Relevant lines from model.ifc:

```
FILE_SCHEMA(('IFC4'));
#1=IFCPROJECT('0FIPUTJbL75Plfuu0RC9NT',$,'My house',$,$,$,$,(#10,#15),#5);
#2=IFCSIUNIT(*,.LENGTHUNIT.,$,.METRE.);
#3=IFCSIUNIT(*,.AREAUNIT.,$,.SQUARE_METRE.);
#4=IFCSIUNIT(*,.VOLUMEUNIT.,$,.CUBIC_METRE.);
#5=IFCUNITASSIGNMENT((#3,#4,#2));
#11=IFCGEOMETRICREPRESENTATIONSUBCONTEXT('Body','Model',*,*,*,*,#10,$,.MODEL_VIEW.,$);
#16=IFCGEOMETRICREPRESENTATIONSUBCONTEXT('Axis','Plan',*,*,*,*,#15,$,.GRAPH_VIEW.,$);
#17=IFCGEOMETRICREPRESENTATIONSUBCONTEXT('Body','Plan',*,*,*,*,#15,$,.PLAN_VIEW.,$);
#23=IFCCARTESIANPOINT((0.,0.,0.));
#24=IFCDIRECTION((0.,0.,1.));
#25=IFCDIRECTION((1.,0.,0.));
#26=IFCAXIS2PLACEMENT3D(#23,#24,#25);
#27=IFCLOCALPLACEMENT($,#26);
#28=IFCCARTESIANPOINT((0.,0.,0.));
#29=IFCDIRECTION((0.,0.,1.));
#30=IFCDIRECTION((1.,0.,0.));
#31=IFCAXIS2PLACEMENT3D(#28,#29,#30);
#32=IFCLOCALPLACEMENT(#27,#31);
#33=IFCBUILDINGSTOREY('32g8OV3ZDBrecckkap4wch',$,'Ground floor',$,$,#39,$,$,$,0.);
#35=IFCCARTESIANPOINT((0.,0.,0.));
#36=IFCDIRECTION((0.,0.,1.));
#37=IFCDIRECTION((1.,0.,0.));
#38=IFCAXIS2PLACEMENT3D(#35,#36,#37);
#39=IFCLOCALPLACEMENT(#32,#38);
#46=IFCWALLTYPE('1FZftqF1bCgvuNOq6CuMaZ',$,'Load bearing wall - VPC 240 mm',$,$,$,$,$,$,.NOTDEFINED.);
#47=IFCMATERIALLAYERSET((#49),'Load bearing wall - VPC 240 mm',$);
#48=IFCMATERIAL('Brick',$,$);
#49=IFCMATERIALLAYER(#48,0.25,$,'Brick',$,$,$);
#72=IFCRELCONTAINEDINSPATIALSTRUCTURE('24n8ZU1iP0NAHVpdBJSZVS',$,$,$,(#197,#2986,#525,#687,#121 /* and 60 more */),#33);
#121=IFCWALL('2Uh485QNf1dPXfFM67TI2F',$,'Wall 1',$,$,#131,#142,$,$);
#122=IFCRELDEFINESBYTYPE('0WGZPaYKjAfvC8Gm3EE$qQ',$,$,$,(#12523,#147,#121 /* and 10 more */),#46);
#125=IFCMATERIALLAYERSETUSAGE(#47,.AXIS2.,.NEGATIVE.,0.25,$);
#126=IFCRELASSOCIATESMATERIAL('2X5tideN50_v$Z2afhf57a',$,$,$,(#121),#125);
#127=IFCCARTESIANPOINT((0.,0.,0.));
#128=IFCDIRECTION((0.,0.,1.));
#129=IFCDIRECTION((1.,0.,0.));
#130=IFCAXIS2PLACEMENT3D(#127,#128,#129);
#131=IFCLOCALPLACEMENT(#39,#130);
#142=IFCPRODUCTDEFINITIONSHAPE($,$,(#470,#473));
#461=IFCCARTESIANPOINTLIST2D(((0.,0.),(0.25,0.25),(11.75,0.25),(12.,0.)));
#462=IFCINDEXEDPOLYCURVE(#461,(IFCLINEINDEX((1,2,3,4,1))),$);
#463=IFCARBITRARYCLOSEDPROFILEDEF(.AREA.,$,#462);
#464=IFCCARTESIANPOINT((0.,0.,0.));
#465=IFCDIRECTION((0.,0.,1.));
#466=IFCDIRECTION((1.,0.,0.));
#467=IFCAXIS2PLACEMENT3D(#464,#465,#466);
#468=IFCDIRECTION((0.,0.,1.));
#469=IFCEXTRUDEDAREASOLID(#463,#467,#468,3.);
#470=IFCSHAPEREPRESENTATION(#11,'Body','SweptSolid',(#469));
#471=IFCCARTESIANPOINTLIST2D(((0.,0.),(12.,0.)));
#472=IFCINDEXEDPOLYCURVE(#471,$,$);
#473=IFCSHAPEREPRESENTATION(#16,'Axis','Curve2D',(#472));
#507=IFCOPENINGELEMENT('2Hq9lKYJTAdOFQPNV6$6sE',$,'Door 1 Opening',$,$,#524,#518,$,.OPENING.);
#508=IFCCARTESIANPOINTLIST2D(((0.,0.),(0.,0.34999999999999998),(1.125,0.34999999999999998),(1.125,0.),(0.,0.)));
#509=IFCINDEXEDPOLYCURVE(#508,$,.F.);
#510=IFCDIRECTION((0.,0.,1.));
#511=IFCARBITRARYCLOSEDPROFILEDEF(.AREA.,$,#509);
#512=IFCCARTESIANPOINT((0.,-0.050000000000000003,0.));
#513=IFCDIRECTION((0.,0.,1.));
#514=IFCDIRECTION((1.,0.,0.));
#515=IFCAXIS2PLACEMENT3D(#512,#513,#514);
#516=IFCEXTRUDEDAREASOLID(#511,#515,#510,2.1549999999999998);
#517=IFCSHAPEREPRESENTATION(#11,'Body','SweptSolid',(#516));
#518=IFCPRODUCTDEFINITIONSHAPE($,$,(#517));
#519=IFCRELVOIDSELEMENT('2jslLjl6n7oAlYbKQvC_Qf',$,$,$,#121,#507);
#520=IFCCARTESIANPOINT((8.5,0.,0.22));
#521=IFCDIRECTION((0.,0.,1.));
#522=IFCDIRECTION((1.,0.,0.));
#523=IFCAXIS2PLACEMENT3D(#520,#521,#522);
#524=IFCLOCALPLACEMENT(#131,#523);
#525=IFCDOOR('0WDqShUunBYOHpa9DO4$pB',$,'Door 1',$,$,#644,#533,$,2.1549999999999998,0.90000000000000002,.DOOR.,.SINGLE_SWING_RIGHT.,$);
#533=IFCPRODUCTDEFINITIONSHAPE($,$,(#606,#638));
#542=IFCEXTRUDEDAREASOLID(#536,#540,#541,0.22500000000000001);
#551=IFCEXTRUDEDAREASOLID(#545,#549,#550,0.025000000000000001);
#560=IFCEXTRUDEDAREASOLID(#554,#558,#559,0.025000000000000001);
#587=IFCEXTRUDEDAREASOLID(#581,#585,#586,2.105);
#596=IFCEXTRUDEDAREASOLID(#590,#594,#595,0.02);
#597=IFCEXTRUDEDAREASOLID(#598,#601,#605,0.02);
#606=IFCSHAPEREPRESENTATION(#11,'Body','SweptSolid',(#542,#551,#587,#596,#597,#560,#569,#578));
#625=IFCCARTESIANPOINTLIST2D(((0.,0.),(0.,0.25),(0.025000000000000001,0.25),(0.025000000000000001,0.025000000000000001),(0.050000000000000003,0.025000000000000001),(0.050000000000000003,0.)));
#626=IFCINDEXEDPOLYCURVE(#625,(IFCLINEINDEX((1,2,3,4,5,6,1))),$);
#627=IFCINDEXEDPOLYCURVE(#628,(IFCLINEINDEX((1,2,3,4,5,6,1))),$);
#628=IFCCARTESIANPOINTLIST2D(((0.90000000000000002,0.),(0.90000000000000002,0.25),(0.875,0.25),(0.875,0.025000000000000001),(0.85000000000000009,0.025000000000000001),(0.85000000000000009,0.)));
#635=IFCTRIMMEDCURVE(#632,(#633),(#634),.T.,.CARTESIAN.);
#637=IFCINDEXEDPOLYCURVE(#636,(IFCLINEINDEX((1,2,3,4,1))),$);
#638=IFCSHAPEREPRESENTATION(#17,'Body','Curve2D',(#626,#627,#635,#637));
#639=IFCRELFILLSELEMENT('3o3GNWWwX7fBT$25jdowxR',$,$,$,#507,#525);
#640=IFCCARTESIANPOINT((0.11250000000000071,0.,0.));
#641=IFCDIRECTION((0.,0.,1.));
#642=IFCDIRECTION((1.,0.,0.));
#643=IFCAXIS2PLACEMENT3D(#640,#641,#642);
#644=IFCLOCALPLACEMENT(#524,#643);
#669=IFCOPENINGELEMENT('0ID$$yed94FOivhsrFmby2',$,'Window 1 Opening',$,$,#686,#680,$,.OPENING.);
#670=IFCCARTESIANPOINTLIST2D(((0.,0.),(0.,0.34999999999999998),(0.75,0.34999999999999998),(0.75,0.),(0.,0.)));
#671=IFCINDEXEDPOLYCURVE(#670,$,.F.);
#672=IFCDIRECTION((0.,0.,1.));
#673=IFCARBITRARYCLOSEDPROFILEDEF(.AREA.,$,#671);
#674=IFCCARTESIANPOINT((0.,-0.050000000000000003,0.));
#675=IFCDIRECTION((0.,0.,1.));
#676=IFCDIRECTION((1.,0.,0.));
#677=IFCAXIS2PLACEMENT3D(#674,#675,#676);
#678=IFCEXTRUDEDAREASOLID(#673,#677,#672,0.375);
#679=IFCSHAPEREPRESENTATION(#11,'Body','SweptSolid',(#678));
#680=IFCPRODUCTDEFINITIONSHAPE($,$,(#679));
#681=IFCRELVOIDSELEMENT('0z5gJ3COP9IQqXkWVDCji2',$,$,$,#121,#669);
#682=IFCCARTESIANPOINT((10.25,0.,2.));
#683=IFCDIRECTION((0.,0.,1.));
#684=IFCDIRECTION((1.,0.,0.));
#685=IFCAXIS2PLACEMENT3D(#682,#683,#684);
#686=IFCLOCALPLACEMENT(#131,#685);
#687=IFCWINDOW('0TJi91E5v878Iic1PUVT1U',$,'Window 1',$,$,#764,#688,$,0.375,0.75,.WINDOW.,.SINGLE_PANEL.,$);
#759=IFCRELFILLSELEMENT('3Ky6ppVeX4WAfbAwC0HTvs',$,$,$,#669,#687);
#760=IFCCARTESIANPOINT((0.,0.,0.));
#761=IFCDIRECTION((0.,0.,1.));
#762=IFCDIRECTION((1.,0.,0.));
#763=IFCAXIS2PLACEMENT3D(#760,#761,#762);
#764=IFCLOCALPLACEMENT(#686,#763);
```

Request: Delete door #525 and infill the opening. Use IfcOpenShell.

```python
import ifcopenshell
import ifcopenshell.api.feature
import ifcopenshell.api.root
import ifcopenshell.geom
import ifcopenshell.util.shape

model = ifcopenshell.open("model.ifc")
settings = ifcopenshell.geom.settings()


def volume(element):
    """Net volume in cubic metres, openings subtracted."""
    shape = ifcopenshell.geom.create_shape(settings, element)
    return ifcopenshell.util.shape.get_volume(shape.geometry)


door = model.by_guid("0WDqShUunBYOHpa9DO4$pB")
opening = door.FillsVoids[0].RelatingOpeningElement
wall = opening.VoidsElements[0].RelatingBuildingElement
before = volume(wall)

ifcopenshell.api.root.remove_product(model, product=door)
ifcopenshell.api.feature.remove_feature(model, feature=opening)

after = volume(wall)

print(f"wall volume {before:.3f} -> {after:.3f} m3")

model.write("model_edited.ifc")
```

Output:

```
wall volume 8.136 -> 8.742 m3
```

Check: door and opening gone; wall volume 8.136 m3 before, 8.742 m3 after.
